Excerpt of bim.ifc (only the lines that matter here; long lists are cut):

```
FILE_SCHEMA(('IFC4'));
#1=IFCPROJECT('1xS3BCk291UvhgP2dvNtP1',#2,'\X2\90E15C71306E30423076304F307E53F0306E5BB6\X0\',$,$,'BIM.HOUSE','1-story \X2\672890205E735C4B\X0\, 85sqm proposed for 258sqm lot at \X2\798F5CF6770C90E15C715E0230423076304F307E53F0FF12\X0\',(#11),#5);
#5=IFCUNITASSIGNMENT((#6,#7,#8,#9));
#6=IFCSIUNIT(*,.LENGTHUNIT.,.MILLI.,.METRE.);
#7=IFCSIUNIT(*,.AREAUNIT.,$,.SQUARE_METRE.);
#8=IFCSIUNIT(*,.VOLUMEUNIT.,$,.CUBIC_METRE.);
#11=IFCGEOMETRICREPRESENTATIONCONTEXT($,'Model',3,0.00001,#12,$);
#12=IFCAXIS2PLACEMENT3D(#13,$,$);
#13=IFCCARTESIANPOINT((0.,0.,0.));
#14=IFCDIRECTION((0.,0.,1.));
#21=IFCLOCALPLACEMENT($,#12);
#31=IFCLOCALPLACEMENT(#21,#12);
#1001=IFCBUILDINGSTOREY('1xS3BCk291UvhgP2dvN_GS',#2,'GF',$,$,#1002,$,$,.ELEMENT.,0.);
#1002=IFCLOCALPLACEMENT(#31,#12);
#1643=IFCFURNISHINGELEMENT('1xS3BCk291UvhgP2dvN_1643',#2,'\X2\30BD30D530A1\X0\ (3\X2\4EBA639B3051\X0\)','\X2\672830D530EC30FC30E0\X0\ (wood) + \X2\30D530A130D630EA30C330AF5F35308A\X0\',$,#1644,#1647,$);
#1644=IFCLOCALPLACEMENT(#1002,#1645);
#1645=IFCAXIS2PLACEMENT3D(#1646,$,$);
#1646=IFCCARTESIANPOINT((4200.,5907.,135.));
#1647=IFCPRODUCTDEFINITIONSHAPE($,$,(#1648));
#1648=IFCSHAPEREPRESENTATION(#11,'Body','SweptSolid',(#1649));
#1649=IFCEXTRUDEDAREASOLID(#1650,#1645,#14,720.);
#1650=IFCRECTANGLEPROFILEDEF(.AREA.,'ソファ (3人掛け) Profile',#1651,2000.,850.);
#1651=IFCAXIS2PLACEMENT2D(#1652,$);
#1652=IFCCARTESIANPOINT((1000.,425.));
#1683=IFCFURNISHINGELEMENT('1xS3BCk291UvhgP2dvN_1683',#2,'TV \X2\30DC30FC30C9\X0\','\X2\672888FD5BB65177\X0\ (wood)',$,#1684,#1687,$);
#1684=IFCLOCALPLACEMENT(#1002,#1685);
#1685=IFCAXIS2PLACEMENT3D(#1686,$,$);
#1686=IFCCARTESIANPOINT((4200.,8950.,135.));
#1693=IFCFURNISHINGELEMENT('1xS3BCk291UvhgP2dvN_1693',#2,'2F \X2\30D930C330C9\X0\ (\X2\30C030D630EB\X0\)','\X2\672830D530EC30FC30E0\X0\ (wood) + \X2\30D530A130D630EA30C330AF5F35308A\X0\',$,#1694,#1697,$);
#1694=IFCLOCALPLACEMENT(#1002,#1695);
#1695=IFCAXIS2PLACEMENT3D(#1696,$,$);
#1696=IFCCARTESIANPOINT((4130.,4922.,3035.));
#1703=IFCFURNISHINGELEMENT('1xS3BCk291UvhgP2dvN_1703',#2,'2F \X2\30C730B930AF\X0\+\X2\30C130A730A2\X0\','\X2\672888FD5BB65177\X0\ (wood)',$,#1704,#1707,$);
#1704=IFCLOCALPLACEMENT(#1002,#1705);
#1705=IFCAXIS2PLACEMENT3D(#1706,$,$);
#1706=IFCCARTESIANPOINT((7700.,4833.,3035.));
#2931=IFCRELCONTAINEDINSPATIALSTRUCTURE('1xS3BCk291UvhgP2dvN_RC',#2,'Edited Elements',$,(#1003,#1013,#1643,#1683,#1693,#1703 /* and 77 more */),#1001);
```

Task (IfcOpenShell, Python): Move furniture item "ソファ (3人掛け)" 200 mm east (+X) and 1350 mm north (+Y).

```python
import ifcopenshell
import ifcopenshell.api.geometry
import ifcopenshell.util.placement
import ifcopenshell.util.unit

model = ifcopenshell.open("bim.ifc")
unit_scale = ifcopenshell.util.unit.calculate_unit_scale(model)

item = model.by_guid("1xS3BCk291UvhgP2dvN_1643")
matrix = ifcopenshell.util.placement.get_local_placement(item.ObjectPlacement)
matrix[0, 3] += 0.2 / unit_scale
matrix[1, 3] += 1.35 / unit_scale
ifcopenshell.api.geometry.edit_object_placement(model, product=item, matrix=matrix, is_si=False)

print(ifcopenshell.util.placement.get_local_placement(item.ObjectPlacement).round(3) + 0.0)

model.write("bim-out.ifc")
```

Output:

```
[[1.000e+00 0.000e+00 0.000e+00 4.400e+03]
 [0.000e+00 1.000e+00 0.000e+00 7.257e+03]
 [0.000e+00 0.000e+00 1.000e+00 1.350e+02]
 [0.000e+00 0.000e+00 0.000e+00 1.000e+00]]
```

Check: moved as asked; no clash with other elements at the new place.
